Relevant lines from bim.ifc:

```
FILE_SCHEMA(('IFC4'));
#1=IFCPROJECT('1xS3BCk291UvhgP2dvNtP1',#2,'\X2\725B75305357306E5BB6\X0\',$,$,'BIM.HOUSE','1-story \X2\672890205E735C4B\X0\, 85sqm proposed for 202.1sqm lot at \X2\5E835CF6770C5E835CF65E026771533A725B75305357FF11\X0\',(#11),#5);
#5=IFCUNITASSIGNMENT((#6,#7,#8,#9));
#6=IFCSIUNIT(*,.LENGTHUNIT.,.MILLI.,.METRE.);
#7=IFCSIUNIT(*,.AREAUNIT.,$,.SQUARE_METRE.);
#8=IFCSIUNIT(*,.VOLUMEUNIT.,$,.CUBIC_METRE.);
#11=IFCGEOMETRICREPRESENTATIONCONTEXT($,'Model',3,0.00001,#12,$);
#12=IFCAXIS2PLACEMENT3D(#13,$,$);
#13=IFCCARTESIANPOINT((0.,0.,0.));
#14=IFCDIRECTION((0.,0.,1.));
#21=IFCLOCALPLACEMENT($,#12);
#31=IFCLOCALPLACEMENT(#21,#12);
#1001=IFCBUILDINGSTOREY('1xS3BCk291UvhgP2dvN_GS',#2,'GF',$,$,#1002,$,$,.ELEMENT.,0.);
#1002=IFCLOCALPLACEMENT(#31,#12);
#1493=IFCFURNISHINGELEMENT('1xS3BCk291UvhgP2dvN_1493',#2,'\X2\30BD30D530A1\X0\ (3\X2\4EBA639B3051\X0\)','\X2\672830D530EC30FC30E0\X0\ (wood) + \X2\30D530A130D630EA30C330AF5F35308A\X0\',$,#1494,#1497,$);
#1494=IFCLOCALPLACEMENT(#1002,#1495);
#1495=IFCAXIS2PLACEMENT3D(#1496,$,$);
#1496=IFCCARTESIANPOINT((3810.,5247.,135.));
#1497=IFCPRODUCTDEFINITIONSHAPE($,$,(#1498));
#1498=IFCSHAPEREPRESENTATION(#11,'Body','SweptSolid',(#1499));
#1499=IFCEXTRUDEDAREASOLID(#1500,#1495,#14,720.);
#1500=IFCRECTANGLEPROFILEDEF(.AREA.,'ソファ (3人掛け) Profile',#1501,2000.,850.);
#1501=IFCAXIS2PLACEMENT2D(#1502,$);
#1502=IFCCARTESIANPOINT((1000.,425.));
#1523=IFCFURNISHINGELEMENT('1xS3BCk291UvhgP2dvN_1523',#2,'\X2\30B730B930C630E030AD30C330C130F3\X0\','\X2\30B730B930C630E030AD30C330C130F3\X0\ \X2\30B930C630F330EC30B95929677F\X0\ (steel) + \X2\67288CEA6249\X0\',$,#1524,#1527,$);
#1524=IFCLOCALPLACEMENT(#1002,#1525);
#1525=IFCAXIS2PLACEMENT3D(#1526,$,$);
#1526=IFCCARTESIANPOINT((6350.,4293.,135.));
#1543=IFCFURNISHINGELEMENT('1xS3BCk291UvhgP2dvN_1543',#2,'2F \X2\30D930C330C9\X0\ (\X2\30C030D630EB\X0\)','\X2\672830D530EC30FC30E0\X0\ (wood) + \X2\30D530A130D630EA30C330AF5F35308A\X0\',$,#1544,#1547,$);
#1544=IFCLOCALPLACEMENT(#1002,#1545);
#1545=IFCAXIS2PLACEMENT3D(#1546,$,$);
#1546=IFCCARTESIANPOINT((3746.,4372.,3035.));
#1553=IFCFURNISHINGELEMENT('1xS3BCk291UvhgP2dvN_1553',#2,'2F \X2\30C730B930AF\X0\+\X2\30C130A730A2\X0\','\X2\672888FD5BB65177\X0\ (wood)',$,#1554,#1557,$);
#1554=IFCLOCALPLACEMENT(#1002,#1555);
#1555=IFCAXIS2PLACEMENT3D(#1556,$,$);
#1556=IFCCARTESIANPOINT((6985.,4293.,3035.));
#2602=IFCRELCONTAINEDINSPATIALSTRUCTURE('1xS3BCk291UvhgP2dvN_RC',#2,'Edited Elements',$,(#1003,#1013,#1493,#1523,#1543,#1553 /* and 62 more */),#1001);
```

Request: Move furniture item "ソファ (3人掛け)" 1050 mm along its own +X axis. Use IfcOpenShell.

```python
import ifcopenshell
import ifcopenshell.api.geometry
import ifcopenshell.util.placement
import ifcopenshell.util.unit

model = ifcopenshell.open("bim.ifc")
unit_scale = ifcopenshell.util.unit.calculate_unit_scale(model)

item = model.by_id(1493)
matrix = ifcopenshell.util.placement.get_local_placement(item.ObjectPlacement)
matrix[:3, 3] += matrix[:3, 0] * 1.05 / unit_scale
ifcopenshell.api.geometry.edit_object_placement(model, product=item, matrix=matrix, is_si=False)

print(ifcopenshell.util.placement.get_local_placement(item.ObjectPlacement).round(3) + 0.0)

model.write("bim_updated.ifc")
```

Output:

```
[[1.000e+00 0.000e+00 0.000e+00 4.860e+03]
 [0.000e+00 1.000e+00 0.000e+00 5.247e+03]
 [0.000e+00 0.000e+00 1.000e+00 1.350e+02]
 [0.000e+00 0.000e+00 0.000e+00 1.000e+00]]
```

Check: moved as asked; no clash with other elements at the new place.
